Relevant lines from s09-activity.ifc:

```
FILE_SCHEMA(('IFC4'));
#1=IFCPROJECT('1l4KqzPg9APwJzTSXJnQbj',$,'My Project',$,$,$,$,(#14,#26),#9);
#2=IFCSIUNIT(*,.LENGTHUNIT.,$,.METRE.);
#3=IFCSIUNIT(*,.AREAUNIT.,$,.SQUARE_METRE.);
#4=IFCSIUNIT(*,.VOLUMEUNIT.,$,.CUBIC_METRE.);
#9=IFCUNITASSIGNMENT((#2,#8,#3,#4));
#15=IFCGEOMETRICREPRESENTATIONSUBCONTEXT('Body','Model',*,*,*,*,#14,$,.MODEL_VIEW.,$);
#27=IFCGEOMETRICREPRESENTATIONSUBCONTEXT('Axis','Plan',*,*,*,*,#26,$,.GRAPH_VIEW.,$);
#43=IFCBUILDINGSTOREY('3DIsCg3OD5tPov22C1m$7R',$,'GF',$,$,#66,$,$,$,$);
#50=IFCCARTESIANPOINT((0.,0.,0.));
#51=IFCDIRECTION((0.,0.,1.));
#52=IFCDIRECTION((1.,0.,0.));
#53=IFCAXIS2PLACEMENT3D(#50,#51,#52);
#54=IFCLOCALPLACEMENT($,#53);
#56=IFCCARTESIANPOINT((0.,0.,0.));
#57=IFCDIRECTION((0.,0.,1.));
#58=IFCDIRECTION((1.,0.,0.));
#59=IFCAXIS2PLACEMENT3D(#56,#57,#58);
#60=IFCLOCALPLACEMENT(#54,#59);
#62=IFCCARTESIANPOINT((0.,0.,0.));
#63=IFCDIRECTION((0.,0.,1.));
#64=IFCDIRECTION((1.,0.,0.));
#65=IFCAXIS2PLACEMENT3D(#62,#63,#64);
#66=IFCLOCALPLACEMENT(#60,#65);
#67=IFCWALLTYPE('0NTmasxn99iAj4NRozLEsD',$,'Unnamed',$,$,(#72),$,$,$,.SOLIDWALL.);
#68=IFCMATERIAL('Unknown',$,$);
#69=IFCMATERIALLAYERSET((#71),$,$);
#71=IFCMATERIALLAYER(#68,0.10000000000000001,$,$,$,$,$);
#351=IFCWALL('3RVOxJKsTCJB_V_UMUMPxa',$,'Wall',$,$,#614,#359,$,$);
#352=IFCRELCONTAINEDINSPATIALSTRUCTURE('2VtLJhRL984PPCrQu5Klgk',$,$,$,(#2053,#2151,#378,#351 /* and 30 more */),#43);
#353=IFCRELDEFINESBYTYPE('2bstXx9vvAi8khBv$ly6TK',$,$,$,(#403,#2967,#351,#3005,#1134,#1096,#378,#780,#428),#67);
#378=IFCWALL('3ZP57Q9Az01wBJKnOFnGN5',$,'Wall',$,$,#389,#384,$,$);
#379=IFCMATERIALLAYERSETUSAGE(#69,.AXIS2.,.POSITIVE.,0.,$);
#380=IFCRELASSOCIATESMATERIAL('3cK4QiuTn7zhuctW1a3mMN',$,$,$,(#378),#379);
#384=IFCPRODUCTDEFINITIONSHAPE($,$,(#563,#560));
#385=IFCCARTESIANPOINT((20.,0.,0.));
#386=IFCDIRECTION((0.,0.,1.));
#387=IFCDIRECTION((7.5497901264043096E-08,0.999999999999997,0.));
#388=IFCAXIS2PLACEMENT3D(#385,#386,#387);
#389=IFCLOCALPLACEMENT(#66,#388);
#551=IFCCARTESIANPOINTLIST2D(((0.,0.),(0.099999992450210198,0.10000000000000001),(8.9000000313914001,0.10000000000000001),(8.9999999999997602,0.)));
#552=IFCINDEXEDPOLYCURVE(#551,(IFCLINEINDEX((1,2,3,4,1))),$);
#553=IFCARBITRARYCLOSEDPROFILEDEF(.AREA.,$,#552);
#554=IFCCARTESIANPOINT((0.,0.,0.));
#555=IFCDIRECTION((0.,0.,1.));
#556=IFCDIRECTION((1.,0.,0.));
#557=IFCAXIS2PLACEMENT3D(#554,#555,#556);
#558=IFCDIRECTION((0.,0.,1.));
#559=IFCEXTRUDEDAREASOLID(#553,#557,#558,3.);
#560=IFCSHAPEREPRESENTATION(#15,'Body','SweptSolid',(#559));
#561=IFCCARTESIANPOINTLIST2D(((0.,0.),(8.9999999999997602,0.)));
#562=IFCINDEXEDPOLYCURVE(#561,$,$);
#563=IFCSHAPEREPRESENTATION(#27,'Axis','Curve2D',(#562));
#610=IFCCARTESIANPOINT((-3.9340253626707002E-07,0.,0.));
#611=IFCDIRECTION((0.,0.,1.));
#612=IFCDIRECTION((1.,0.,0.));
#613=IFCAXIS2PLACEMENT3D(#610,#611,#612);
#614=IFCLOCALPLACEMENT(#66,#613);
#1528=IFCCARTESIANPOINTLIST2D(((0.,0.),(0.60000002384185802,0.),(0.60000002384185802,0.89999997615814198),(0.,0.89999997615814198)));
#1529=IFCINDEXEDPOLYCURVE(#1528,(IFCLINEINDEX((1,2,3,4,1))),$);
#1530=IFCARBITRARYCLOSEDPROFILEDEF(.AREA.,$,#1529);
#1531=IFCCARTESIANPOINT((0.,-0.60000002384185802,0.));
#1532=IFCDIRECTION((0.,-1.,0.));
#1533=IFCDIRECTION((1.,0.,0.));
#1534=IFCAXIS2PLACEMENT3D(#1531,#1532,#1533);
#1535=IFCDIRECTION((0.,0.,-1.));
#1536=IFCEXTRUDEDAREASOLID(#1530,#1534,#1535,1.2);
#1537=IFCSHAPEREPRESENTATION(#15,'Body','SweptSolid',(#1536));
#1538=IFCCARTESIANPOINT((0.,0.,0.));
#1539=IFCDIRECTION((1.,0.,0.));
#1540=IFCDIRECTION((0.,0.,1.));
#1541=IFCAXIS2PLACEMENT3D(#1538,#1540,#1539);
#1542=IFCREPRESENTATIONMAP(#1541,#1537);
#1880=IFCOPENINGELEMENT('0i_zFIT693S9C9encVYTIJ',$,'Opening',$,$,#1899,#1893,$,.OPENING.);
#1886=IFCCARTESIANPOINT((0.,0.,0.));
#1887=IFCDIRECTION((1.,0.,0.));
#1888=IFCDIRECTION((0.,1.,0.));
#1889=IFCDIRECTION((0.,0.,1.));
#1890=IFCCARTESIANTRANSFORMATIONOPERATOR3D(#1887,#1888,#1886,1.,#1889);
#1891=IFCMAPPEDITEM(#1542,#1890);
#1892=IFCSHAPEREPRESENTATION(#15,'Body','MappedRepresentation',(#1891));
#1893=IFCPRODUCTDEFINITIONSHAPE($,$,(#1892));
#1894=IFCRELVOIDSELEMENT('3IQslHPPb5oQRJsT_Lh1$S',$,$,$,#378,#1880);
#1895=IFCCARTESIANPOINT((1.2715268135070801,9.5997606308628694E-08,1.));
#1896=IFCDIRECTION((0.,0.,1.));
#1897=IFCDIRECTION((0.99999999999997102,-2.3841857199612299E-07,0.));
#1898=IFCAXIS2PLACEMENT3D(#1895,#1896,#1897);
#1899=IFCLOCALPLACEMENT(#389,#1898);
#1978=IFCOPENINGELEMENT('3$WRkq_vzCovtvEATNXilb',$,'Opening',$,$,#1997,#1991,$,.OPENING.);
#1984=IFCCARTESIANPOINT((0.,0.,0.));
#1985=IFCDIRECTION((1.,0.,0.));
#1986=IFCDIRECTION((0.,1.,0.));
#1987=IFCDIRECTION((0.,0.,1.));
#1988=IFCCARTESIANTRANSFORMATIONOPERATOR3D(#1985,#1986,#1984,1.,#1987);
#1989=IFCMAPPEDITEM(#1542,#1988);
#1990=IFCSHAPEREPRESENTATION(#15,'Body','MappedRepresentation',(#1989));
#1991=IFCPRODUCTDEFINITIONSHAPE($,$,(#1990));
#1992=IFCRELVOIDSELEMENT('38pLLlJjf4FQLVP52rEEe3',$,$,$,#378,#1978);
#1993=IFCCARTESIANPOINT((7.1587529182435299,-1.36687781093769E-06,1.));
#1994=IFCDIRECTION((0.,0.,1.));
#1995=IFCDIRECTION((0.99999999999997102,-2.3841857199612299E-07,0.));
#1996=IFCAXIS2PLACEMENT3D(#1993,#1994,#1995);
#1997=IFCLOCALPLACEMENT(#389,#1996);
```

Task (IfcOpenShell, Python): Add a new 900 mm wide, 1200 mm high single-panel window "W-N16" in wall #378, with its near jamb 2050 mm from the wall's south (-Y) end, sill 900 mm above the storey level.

```python
import numpy as np
import ifcopenshell
import ifcopenshell.api.feature
import ifcopenshell.api.geometry
import ifcopenshell.api.root
import ifcopenshell.api.spatial
import ifcopenshell.geom
import ifcopenshell.util.element
import ifcopenshell.util.placement
import ifcopenshell.util.representation
import ifcopenshell.util.shape
import ifcopenshell.util.unit

model = ifcopenshell.open("s09-activity.ifc")
unit_scale = ifcopenshell.util.unit.calculate_unit_scale(model)
settings = ifcopenshell.geom.settings()


def volume(element):
    """Net volume in cubic metres, openings subtracted."""
    shape = ifcopenshell.geom.create_shape(settings, element)
    return ifcopenshell.util.shape.get_volume(shape.geometry)


wall = model.by_guid("3ZP57Q9Az01wBJKnOFnGN5")
storey = ifcopenshell.util.element.get_container(wall, ifc_class="IfcBuildingStorey")
context = ifcopenshell.util.representation.get_context(model, "Model", "Body", "MODEL_VIEW")
before = volume(wall)

width, height, from_end, sill = 0.9, 1.2, 2.05, 0.9  # metres

# The wall runs along its own X axis, and the end named is its -X end.
wall_shape = ifcopenshell.geom.create_shape(settings, wall)
x, y, z = ifcopenshell.util.shape.get_vertices(wall_shape.geometry).T
start = x.min() + from_end
face, thickness = float(y.min()), float(y.max() - y.min())
wall_matrix = ifcopenshell.util.placement.get_local_placement(wall.ObjectPlacement)
level = ifcopenshell.util.placement.get_local_placement(storey.ObjectPlacement)[2, 3]


def in_wall(x, y):
    """Placement at x, y metres in the wall's axes, at sill height."""
    matrix = wall_matrix.copy()
    matrix[:, 3] = wall_matrix @ np.array([x / unit_scale, y / unit_scale, 0.0, 1.0])
    matrix[2, 3] = level + sill / unit_scale
    return matrix


# Opening: a box that overshoots both wall faces by 50 mm.
opening = ifcopenshell.api.root.create_entity(model, ifc_class="IfcOpeningElement", predefined_type="OPENING")
box = ifcopenshell.api.geometry.add_wall_representation(
    model, context=context, length=width, height=height, thickness=thickness + 0.1
)
ifcopenshell.api.geometry.assign_representation(model, product=opening, representation=box)
ifcopenshell.api.geometry.edit_object_placement(model, product=opening, matrix=in_wall(start, face - 0.05), is_si=False)
ifcopenshell.api.feature.add_feature(model, feature=opening, element=wall)

window = ifcopenshell.api.root.create_entity(model, ifc_class="IfcWindow", name="W-N16", predefined_type="WINDOW")
window.OverallWidth, window.OverallHeight = width / unit_scale, height / unit_scale
window.PartitioningType = "SINGLE_PANEL"
body = ifcopenshell.api.geometry.add_window_representation(
    model,
    context=context,
    overall_width=window.OverallWidth,
    overall_height=window.OverallHeight,
    partition_type="SINGLE_PANEL",
)
ifcopenshell.api.geometry.assign_representation(model, product=window, representation=body)
ifcopenshell.api.spatial.assign_container(model, products=[window], relating_structure=storey)
ifcopenshell.api.feature.add_filling(model, opening=opening, element=window)

# Centre the window in the wall's thickness.
ifcopenshell.api.geometry.edit_object_placement(model, product=window, matrix=in_wall(start, face), is_si=False)
window_shape = ifcopenshell.geom.create_shape(settings, window)
depth = ifcopenshell.util.shape.get_vertices(window_shape.geometry)[:, 1]
offset = face + thickness / 2 - (depth.min() + depth.max()) / 2
ifcopenshell.api.geometry.edit_object_placement(model, product=window, matrix=in_wall(start, offset), is_si=False)

after = volume(wall)

print(f"wall volume {before:.3f} -> {after:.3f} m3")

model.write("s09-activity_updated.ifc")
```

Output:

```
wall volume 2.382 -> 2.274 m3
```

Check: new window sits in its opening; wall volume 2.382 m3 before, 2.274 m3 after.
